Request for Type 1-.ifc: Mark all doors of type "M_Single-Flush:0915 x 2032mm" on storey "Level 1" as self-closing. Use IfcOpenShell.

First a look at what the model holds.

```python
import ifcopenshell
import ifcopenshell.util.element

model = ifcopenshell.open("Type 1-.ifc")
print(model.schema)
storey = next(s for s in model.by_type("IfcBuildingStorey") if s.Name == "Level 1")
doors = [e for e in ifcopenshell.util.element.get_decomposition(storey) if e.is_a("IfcDoor")]
seen = {}
for e in doors:
    element_type = ifcopenshell.util.element.get_type(e)
    key = (element_type.Name if element_type != e and element_type else None, ifcopenshell.util.element.get_pset(e, "Pset_DoorCommon", "SelfClosing"))
    seen[key] = seen.get(key, 0) + 1
for (name, value), count in sorted(seen.items(), key=str):
    print(count, "x", name, "|", value)
```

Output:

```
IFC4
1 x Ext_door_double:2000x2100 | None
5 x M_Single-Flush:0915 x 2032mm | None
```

```python
import ifcopenshell
import ifcopenshell.api.pset
import ifcopenshell.util.element

model = ifcopenshell.open("Type 1-.ifc")

storey = next(s for s in model.by_type("IfcBuildingStorey") if s.Name == "Level 1")
doors = [e for e in ifcopenshell.util.element.get_decomposition(storey) if e.is_a("IfcDoor")]

count = 0
for e in doors:
    element_type = ifcopenshell.util.element.get_type(e)
    if element_type in (None, e) or element_type.Name != "M_Single-Flush:0915 x 2032mm":
        continue
    # add_pset returns the element's existing set when there is one.
    pset = ifcopenshell.api.pset.add_pset(model, product=e, name="Pset_DoorCommon")
    ifcopenshell.api.pset.edit_pset(model, pset=pset, properties={"SelfClosing": True})
    count += 1

print(count, "doors updated")

model.write("Type 1-_updated.ifc")
```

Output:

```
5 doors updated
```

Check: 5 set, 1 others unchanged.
